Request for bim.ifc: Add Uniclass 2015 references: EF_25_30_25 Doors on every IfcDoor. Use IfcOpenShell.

First a look at what the model holds.

```python
import ifcopenshell

model = ifcopenshell.open("bim.ifc")
print(model.schema)
print("classifications:", [c.Name for c in model.by_type("IfcClassification")])
for ifc_class in ("IfcDoor", "IfcRoof", "IfcStair", "IfcWall", "IfcWindow"):
    print(ifc_class, len(model.by_type(ifc_class)))
```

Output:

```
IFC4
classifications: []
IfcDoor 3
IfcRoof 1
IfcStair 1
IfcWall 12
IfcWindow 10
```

```python
import ifcopenshell
import ifcopenshell.api.classification

model = ifcopenshell.open("bim.ifc")

system = ifcopenshell.api.classification.add_classification(model, classification="Uniclass 2015")

codes = {
    "IfcDoor": ("EF_25_30_25", "Doors"),
}
for ifc_class, (code, name) in codes.items():
    products = model.by_type(ifc_class)
    ifcopenshell.api.classification.add_reference(
        model, products=products, classification=system, identification=code, name=name
    )
    print(code, len(products))

model.write("bim-out.ifc")
```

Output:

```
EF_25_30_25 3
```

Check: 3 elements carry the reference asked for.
